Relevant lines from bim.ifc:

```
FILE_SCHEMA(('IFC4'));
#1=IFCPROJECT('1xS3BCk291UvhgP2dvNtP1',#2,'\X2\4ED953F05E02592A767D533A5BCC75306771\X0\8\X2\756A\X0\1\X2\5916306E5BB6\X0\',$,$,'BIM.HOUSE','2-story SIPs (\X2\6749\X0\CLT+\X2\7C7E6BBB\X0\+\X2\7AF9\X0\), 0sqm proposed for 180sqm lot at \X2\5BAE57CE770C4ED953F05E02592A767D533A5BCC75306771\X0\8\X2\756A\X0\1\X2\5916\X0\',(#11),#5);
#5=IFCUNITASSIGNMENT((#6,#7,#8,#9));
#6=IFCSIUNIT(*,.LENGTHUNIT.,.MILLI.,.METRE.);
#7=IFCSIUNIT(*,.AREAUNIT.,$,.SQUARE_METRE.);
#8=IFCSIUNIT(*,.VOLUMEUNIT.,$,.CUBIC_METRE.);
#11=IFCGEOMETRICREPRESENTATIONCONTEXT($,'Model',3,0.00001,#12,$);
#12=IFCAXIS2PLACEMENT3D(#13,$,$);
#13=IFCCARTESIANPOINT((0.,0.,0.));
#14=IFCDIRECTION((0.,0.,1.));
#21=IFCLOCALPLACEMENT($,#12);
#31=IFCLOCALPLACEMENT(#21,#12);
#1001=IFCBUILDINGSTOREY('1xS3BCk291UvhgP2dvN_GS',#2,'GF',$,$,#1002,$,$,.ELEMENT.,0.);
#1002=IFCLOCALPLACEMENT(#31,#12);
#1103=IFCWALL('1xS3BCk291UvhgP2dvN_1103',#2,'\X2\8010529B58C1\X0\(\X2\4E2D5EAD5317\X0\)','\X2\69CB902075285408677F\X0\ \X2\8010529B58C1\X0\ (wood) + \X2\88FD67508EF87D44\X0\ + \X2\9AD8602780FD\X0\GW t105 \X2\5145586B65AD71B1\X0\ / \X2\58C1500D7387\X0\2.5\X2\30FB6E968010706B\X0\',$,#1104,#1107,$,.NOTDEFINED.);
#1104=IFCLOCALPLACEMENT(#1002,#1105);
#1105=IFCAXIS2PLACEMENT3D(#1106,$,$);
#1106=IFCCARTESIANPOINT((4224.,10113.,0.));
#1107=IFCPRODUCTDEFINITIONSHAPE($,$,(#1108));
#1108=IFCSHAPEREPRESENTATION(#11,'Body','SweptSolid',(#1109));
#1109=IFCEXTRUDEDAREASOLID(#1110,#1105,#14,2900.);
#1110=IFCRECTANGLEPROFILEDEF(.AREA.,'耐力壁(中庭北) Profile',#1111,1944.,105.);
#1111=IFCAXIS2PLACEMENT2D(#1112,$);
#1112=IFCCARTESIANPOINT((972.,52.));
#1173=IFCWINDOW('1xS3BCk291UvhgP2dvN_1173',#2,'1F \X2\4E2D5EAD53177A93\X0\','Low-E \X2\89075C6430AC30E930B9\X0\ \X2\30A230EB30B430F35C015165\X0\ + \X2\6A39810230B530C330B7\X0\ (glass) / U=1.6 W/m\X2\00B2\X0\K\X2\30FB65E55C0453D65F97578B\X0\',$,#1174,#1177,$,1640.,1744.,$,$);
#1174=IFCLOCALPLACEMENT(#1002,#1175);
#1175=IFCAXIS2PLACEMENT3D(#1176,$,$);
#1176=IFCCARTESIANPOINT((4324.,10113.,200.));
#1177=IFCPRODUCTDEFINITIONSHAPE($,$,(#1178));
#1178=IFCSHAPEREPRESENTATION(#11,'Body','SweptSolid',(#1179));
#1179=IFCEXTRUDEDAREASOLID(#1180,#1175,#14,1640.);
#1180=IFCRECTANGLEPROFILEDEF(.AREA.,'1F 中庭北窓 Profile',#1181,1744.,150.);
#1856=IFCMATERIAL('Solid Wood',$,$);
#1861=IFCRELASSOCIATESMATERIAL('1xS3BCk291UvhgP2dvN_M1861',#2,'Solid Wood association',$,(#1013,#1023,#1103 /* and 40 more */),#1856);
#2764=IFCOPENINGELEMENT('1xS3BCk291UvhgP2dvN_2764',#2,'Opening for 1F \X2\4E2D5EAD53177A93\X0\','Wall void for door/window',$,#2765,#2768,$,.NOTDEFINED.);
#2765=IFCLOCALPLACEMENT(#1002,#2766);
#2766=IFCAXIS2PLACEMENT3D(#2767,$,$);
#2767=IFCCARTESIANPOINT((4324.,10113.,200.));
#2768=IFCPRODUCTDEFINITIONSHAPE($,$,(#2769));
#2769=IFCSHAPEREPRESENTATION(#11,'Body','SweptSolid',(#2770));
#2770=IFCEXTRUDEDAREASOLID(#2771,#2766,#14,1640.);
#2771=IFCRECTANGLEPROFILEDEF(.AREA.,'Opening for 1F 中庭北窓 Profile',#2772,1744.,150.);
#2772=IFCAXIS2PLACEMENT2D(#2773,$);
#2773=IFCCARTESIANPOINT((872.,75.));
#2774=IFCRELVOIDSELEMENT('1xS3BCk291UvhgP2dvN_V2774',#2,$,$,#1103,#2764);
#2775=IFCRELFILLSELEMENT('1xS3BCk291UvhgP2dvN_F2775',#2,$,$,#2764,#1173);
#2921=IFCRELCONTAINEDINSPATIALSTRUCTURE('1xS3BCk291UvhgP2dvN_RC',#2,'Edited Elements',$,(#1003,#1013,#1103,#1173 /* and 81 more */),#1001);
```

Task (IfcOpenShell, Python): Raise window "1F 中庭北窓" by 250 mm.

```python
import numpy as np
import ifcopenshell
import ifcopenshell.api.geometry
import ifcopenshell.util.placement
import ifcopenshell.util.unit

model = ifcopenshell.open("bim.ifc")
unit_scale = ifcopenshell.util.unit.calculate_unit_scale(model)

window = model.by_id(1173)
opening = window.FillsVoids[0].RelatingOpeningElement
dz = 250.0

shift = np.array([0.0, 0.0, dz])
# The window is not placed relative to its opening, so move both.
for product in (opening, window):
    matrix = ifcopenshell.util.placement.get_local_placement(product.ObjectPlacement)
    matrix[:3, 3] += shift
    ifcopenshell.api.geometry.edit_object_placement(model, product=product, matrix=matrix, is_si=False)

print(f"moved by {dz * unit_scale:+.3f} m")

model.write("bim_updated.ifc")
```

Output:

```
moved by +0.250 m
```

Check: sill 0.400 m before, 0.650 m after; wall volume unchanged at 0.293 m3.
